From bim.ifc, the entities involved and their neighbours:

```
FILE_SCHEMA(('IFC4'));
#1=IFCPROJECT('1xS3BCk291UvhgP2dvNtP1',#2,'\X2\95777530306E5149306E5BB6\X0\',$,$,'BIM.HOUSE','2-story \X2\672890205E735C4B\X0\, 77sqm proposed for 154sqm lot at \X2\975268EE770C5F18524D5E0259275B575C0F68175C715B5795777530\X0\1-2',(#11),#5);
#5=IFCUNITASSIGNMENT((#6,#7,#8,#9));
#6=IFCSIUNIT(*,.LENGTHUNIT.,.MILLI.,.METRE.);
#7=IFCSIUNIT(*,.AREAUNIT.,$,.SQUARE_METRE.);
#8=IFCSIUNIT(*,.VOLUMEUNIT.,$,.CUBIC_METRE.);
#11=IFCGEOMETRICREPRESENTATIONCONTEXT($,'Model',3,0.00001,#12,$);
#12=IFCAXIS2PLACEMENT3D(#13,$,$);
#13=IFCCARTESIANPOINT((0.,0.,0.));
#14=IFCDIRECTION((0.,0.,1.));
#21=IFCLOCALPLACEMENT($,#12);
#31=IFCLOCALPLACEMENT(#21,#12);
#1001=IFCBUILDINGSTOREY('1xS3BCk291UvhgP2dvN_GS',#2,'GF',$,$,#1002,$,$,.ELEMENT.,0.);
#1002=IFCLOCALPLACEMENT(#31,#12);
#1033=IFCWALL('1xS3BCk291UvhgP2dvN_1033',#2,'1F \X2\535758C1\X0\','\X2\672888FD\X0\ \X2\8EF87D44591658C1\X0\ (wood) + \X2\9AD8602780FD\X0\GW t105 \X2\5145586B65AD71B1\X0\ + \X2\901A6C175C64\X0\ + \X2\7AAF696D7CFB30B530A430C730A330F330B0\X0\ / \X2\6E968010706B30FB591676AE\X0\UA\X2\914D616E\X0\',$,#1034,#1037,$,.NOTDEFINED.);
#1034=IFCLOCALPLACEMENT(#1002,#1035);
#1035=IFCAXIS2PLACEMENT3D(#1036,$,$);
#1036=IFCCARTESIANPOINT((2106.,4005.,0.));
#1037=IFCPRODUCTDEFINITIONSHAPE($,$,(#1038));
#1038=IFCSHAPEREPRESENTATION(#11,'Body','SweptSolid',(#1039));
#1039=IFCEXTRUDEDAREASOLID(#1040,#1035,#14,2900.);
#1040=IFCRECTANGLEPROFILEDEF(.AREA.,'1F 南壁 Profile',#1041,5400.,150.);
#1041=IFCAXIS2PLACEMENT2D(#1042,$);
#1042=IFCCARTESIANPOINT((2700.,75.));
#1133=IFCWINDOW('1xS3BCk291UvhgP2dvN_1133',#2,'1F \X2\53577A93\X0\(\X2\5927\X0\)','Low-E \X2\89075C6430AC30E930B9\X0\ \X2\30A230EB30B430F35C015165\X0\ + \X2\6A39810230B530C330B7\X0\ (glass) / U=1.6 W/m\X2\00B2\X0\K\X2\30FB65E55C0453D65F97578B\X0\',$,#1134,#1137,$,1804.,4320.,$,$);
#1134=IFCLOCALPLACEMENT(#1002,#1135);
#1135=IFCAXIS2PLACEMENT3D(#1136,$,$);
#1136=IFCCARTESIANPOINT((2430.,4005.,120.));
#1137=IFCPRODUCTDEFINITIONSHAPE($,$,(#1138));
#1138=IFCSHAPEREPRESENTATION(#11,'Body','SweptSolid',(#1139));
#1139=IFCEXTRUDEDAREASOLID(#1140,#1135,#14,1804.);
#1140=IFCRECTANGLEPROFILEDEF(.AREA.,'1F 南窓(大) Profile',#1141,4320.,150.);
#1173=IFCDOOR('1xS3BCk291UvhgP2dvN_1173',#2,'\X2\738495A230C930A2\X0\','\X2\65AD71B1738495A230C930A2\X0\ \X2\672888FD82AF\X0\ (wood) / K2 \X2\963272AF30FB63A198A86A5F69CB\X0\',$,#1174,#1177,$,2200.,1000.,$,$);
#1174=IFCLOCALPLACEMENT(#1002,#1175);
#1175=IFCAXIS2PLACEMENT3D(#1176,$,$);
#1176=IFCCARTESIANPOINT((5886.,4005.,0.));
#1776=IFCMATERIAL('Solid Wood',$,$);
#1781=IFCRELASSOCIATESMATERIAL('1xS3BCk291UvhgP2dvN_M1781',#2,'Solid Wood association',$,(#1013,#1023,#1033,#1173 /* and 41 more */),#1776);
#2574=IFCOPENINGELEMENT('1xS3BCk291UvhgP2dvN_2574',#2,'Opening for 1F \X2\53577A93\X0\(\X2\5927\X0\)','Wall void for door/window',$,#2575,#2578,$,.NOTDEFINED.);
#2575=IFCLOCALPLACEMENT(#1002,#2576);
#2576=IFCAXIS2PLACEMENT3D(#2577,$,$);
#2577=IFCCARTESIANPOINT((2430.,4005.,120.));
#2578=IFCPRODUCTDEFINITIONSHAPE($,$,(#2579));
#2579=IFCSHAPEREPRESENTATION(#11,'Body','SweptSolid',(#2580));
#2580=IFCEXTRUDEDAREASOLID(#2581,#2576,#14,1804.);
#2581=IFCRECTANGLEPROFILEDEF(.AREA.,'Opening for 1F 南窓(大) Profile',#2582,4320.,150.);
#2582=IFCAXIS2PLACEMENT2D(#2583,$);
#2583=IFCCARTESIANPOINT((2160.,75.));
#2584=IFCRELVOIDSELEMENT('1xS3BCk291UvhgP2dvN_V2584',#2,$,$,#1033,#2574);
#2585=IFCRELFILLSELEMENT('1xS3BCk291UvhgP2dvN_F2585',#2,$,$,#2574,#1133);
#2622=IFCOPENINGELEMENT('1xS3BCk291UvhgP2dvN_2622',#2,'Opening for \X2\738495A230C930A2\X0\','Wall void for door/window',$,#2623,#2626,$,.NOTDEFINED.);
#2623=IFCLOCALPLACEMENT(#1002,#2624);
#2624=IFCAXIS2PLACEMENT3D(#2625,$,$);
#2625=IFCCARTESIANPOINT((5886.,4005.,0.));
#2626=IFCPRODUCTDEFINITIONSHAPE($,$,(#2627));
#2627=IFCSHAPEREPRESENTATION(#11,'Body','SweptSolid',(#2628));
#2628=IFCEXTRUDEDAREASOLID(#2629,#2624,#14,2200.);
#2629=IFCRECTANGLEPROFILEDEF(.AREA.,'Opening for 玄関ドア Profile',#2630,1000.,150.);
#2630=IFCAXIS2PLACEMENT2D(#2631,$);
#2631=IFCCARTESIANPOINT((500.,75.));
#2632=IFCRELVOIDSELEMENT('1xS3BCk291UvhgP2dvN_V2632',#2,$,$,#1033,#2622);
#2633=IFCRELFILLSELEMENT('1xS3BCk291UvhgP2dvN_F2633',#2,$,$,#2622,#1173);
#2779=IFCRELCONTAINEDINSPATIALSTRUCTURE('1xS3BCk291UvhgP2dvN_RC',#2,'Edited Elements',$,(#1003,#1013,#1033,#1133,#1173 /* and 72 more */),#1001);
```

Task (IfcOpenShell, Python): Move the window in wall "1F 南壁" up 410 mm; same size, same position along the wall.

```python
import numpy as np
import ifcopenshell
import ifcopenshell.api.geometry
import ifcopenshell.util.placement
import ifcopenshell.util.unit

model = ifcopenshell.open("bim.ifc")
unit_scale = ifcopenshell.util.unit.calculate_unit_scale(model)

window = model.by_guid("1xS3BCk291UvhgP2dvN_1133")
opening = window.FillsVoids[0].RelatingOpeningElement
dz = 410.0

shift = np.array([0.0, 0.0, dz])
# The window is not placed relative to its opening, so move both.
for product in (opening, window):
    matrix = ifcopenshell.util.placement.get_local_placement(product.ObjectPlacement)
    matrix[:3, 3] += shift
    ifcopenshell.api.geometry.edit_object_placement(model, product=product, matrix=matrix, is_si=False)

print(f"moved by {dz * unit_scale:+.3f} m")

model.write("bim_rev.ifc")
```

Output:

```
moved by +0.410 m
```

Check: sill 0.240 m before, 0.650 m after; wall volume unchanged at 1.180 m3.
